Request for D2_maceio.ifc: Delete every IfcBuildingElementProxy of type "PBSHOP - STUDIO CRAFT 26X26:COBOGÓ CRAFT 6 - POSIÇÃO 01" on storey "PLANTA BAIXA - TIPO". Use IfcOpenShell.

First a look at what the model holds.

```python
import ifcopenshell
import ifcopenshell.util.element

model = ifcopenshell.open("D2_maceio.ifc")
print(model.schema)
storey = next(s for s in model.by_type("IfcBuildingStorey") if s.Name == "PLANTA BAIXA - TIPO")
proxies = [e for e in ifcopenshell.util.element.get_decomposition(storey) if e.is_a("IfcBuildingElementProxy")]
seen = {}
for e in proxies:
    element_type = ifcopenshell.util.element.get_type(e)
    name = element_type.Name if element_type not in (None, e) else None
    seen[name] = seen.get(name, 0) + 1
for name, count in sorted(seen.items(), key=str):
    print(count, "x", name)
```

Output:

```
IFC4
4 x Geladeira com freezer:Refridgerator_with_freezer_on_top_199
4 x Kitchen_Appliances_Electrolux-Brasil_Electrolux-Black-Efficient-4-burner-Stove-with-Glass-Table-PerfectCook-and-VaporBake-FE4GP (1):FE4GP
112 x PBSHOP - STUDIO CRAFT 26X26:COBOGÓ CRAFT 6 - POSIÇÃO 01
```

```python
import ifcopenshell
import ifcopenshell.api.root
import ifcopenshell.util.element

model = ifcopenshell.open("D2_maceio.ifc")

storey = next(s for s in model.by_type("IfcBuildingStorey") if s.Name == "PLANTA BAIXA - TIPO")
proxies = [e for e in ifcopenshell.util.element.get_decomposition(storey) if e.is_a("IfcBuildingElementProxy")]
targets = [e for e in proxies if (t := ifcopenshell.util.element.get_type(e)) not in (None, e) and t.Name == "PBSHOP - STUDIO CRAFT 26X26:COBOGÓ CRAFT 6 - POSIÇÃO 01"]

for e in targets:
    ifcopenshell.api.root.remove_product(model, product=e)
print(len(targets), "removed")

model.write("D2_maceio_rev.ifc")
```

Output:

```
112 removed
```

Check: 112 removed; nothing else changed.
